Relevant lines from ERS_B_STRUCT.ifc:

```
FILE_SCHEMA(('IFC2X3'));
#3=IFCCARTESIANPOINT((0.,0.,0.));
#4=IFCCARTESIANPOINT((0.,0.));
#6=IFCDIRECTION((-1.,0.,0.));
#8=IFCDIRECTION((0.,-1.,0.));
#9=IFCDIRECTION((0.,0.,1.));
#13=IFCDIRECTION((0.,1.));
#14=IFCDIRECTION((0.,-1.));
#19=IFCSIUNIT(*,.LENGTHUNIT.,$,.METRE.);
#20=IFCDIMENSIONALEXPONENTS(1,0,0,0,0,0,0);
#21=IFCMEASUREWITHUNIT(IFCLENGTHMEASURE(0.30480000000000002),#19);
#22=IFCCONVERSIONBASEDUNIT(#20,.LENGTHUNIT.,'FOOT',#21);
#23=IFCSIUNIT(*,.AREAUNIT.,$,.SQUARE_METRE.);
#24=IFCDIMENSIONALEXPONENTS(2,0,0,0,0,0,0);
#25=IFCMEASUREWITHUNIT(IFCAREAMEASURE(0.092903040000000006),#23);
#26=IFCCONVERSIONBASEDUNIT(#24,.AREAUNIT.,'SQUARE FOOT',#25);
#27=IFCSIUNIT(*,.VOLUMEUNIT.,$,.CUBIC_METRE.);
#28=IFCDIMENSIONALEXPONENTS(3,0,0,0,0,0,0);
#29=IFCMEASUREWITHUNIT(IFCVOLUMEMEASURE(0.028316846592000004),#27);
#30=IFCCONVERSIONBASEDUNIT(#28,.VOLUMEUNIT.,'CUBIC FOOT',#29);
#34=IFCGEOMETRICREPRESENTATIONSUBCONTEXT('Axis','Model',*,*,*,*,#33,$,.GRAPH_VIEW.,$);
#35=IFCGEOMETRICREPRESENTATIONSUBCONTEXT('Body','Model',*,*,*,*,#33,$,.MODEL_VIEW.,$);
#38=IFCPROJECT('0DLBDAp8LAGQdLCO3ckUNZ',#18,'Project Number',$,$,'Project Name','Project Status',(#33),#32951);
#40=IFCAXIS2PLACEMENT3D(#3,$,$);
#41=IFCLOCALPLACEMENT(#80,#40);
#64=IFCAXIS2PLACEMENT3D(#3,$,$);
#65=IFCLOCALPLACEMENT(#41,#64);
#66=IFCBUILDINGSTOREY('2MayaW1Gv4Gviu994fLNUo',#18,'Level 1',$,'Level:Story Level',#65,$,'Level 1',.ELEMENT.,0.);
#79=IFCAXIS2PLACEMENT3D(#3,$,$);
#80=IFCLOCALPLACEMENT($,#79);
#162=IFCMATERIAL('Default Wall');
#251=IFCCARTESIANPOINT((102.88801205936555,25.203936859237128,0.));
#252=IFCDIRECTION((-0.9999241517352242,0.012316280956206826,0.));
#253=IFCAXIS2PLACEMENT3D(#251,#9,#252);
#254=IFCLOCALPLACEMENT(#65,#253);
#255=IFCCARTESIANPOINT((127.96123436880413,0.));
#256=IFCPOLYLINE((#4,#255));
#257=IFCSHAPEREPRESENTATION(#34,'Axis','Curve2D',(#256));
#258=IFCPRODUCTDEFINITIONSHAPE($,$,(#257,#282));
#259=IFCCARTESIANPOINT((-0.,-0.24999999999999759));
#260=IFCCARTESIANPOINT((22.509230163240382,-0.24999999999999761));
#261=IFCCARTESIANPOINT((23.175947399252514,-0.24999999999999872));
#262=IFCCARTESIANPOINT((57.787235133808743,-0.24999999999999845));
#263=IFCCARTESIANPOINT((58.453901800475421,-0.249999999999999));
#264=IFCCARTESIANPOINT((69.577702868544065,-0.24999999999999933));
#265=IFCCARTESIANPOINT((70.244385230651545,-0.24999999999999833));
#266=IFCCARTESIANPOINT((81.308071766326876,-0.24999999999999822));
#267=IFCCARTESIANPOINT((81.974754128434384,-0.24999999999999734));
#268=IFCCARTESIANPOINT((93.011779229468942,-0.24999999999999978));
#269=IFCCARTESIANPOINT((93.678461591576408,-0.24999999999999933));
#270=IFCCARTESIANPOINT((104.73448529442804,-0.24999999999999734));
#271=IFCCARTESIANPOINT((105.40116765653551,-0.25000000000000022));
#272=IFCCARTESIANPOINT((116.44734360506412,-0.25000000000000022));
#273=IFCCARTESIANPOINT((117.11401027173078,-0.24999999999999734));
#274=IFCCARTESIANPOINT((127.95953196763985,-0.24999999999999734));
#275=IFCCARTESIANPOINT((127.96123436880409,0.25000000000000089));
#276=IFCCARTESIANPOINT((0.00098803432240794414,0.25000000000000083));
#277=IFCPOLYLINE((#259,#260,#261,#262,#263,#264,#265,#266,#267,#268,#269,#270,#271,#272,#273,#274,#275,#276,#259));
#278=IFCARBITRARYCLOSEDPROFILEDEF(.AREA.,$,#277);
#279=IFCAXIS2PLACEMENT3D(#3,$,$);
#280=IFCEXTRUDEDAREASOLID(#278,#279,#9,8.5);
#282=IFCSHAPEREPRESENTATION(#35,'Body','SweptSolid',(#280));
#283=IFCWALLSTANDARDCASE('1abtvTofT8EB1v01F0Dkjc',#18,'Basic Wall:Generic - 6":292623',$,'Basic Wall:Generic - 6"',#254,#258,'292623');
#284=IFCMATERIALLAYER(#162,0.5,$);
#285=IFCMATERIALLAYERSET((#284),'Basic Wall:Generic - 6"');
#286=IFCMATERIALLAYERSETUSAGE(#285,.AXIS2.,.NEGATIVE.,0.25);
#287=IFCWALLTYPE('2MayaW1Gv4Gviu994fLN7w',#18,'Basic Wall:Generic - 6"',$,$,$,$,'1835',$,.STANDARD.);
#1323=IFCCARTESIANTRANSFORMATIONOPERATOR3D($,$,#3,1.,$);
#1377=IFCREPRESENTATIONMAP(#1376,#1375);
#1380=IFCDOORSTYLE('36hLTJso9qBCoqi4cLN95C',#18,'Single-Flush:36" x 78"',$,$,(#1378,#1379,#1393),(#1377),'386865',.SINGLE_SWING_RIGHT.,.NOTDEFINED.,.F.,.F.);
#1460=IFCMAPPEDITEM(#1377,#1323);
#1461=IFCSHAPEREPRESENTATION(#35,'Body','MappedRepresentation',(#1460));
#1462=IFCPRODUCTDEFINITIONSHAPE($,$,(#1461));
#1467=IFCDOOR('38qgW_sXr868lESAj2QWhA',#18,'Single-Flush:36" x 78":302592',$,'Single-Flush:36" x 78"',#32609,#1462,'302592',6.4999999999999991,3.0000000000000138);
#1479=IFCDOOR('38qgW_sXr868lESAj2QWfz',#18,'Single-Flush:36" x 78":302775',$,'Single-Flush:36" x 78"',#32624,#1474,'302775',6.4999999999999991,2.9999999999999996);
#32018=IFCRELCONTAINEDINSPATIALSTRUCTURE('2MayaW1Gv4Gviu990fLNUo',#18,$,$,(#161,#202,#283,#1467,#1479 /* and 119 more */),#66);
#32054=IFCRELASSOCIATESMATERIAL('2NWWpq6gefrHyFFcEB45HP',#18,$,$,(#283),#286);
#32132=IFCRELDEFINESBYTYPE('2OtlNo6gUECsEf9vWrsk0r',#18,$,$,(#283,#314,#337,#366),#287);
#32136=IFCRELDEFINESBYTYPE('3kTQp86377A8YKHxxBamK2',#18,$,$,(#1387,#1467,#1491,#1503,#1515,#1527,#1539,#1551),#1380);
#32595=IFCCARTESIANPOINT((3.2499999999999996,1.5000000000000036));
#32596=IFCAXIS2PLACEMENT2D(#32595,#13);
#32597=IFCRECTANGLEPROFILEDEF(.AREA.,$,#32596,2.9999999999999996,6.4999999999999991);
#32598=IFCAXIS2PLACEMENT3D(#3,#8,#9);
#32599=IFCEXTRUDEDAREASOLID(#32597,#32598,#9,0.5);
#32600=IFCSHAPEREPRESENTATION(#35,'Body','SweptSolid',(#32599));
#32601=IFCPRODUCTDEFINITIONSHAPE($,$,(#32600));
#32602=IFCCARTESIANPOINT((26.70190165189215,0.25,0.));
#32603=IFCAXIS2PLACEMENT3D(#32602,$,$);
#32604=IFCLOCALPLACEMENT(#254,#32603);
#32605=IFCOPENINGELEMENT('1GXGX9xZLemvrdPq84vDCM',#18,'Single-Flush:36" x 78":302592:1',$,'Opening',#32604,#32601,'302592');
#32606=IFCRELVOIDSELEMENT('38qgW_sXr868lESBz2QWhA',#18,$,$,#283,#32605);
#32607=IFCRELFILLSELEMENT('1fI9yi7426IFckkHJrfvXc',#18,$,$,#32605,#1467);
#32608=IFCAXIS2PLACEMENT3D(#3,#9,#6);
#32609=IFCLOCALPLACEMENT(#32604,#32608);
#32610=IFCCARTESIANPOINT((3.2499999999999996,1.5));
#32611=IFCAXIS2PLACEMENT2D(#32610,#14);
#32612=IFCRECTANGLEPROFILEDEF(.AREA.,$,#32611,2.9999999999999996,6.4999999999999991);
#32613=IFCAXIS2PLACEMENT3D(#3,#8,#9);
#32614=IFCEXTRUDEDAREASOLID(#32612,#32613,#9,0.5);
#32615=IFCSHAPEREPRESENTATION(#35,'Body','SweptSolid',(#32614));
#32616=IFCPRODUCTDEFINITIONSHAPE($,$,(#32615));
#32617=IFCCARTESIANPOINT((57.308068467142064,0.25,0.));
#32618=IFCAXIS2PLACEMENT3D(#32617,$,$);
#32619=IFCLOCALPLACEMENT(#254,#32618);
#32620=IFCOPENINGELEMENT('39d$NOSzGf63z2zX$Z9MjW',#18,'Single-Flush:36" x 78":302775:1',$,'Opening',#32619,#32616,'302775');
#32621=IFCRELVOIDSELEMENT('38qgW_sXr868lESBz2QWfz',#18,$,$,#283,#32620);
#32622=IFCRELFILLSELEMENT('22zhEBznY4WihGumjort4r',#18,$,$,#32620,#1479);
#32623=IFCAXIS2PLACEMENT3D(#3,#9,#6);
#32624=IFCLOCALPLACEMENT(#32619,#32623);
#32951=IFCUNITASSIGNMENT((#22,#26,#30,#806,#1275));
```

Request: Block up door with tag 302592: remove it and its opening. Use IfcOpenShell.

```python
import ifcopenshell
import ifcopenshell.api.feature
import ifcopenshell.api.root
import ifcopenshell.geom
import ifcopenshell.util.shape

model = ifcopenshell.open("ERS_B_STRUCT.ifc")
settings = ifcopenshell.geom.settings()


def volume(element):
    """Net volume in cubic metres, openings subtracted."""
    shape = ifcopenshell.geom.create_shape(settings, element)
    return ifcopenshell.util.shape.get_volume(shape.geometry)


door = model.by_guid("38qgW_sXr868lESAj2QWhA")
opening = door.FillsVoids[0].RelatingOpeningElement
wall = opening.VoidsElements[0].RelatingBuildingElement
before = volume(wall)

ifcopenshell.api.root.remove_product(model, product=door)
ifcopenshell.api.feature.remove_feature(model, feature=opening)

after = volume(wall)

print(f"wall volume {before:.3f} -> {after:.3f} m3")

model.write("ERS_B_STRUCT_updated.ifc")
```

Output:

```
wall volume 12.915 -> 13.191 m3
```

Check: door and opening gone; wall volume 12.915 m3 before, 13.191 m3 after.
